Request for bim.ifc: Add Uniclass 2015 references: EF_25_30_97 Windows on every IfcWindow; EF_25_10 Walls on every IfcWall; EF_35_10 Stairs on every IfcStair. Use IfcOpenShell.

First a look at what the model holds.

```python
import ifcopenshell

model = ifcopenshell.open("bim.ifc")
print(model.schema)
print("classifications:", [c.Name for c in model.by_type("IfcClassification")])
for ifc_class in ("IfcDoor", "IfcRoof", "IfcStair", "IfcWall", "IfcWindow"):
    print(ifc_class, len(model.by_type(ifc_class)))
```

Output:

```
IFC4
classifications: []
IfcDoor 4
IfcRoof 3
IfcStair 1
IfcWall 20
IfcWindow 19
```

```python
import ifcopenshell
import ifcopenshell.api.classification

model = ifcopenshell.open("bim.ifc")

system = ifcopenshell.api.classification.add_classification(model, classification="Uniclass 2015")

codes = {
    "IfcWindow": ("EF_25_30_97", "Windows"),
    "IfcWall": ("EF_25_10", "Walls"),
    "IfcStair": ("EF_35_10", "Stairs"),
}
for ifc_class, (code, name) in codes.items():
    products = model.by_type(ifc_class)
    ifcopenshell.api.classification.add_reference(
        model, products=products, classification=system, identification=code, name=name
    )
    print(code, len(products))

model.write("bim_rev.ifc")
```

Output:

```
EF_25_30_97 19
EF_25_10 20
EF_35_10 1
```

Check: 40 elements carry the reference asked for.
